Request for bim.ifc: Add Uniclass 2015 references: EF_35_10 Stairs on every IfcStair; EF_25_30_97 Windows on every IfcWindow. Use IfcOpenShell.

First a look at what the model holds.

```python
import ifcopenshell

model = ifcopenshell.open("bim.ifc")
print(model.schema)
print("classifications:", [c.Name for c in model.by_type("IfcClassification")])
for ifc_class in ("IfcDoor", "IfcRoof", "IfcStair", "IfcWall", "IfcWindow"):
    print(ifc_class, len(model.by_type(ifc_class)))
```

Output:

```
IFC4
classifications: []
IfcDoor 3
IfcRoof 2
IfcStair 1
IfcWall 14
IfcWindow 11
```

```python
import ifcopenshell
import ifcopenshell.api.classification

model = ifcopenshell.open("bim.ifc")

system = ifcopenshell.api.classification.add_classification(model, classification="Uniclass 2015")

codes = {
    "IfcStair": ("EF_35_10", "Stairs"),
    "IfcWindow": ("EF_25_30_97", "Windows"),
}
for ifc_class, (code, name) in codes.items():
    products = model.by_type(ifc_class)
    ifcopenshell.api.classification.add_reference(
        model, products=products, classification=system, identification=code, name=name
    )
    print(code, len(products))

model.write("bim_updated.ifc")
```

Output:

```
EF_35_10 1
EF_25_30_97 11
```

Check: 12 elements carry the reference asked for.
